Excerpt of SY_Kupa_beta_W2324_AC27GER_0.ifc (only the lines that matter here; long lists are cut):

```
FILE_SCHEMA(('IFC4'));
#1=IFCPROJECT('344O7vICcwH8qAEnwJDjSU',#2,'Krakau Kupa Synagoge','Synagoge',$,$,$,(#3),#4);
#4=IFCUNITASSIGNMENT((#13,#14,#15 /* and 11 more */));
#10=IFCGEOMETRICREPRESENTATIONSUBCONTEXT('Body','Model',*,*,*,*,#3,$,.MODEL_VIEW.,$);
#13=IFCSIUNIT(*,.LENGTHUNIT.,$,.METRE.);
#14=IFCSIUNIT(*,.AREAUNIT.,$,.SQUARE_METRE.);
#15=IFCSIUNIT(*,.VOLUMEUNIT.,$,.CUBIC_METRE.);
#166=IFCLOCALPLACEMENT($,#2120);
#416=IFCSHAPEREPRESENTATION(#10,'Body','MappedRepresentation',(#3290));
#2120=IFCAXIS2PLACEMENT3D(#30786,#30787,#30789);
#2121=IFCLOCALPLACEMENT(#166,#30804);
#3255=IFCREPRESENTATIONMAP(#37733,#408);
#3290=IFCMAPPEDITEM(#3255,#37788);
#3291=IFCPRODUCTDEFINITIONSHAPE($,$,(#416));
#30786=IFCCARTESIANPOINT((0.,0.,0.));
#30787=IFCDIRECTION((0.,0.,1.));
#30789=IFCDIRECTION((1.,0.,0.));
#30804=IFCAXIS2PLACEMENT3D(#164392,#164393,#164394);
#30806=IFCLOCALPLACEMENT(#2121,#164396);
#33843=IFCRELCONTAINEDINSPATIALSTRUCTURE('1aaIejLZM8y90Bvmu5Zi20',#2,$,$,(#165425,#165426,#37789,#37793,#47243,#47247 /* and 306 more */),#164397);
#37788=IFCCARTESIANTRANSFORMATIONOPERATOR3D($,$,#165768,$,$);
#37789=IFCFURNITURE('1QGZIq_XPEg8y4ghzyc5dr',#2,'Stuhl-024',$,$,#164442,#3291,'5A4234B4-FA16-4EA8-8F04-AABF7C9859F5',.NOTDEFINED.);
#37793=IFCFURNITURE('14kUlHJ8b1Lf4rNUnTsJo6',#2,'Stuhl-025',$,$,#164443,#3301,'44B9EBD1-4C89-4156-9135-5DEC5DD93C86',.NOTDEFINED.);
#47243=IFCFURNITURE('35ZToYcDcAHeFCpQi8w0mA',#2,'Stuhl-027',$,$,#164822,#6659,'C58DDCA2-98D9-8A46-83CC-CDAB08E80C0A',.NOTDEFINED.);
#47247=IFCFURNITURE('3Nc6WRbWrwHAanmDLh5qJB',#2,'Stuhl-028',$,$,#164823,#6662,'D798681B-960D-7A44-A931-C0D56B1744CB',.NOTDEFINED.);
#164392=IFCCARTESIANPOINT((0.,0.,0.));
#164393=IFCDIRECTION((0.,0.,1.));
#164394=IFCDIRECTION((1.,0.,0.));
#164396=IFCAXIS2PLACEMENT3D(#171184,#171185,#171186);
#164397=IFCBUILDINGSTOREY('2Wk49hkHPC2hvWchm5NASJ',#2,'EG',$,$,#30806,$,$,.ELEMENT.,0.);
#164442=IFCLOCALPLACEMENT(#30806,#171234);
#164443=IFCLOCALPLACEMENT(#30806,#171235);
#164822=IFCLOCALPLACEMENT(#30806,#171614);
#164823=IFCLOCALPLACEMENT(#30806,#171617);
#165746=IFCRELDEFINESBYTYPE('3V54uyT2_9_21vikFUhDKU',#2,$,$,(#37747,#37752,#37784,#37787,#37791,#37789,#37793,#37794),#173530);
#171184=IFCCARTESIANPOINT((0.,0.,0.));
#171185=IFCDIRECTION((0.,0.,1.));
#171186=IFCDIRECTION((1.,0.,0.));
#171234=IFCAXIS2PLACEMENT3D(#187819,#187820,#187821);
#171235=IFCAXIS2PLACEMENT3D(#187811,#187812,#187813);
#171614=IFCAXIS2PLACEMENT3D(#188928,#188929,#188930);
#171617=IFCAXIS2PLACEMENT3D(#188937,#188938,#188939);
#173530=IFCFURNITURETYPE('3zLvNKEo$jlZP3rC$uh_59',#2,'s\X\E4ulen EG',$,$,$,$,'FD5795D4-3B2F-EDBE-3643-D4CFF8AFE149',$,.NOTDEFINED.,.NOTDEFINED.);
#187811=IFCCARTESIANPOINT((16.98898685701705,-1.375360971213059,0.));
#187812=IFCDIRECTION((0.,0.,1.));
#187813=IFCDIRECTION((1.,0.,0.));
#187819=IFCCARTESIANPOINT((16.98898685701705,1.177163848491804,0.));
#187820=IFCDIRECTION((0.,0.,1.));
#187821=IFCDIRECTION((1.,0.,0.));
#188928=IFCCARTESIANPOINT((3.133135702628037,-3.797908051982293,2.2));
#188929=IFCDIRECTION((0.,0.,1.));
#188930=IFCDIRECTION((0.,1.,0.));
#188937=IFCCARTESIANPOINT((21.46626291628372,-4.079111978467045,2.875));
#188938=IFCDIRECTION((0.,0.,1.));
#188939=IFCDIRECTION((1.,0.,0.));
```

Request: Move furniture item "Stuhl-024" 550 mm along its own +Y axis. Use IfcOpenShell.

```python
import ifcopenshell
import ifcopenshell.api.geometry
import ifcopenshell.util.placement
import ifcopenshell.util.unit

model = ifcopenshell.open("SY_Kupa_beta_W2324_AC27GER_0.ifc")
unit_scale = ifcopenshell.util.unit.calculate_unit_scale(model)

item = model.by_guid("1QGZIq_XPEg8y4ghzyc5dr")
matrix = ifcopenshell.util.placement.get_local_placement(item.ObjectPlacement)
matrix[:3, 3] += matrix[:3, 1] * 0.55 / unit_scale
ifcopenshell.api.geometry.edit_object_placement(model, product=item, matrix=matrix, is_si=False)

print(ifcopenshell.util.placement.get_local_placement(item.ObjectPlacement).round(3) + 0.0)

model.write("SY_Kupa_beta_W2324_AC27GER_0_updated.ifc")
```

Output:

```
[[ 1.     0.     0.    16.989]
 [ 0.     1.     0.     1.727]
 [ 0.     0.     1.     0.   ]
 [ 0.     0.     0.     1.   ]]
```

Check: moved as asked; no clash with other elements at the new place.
